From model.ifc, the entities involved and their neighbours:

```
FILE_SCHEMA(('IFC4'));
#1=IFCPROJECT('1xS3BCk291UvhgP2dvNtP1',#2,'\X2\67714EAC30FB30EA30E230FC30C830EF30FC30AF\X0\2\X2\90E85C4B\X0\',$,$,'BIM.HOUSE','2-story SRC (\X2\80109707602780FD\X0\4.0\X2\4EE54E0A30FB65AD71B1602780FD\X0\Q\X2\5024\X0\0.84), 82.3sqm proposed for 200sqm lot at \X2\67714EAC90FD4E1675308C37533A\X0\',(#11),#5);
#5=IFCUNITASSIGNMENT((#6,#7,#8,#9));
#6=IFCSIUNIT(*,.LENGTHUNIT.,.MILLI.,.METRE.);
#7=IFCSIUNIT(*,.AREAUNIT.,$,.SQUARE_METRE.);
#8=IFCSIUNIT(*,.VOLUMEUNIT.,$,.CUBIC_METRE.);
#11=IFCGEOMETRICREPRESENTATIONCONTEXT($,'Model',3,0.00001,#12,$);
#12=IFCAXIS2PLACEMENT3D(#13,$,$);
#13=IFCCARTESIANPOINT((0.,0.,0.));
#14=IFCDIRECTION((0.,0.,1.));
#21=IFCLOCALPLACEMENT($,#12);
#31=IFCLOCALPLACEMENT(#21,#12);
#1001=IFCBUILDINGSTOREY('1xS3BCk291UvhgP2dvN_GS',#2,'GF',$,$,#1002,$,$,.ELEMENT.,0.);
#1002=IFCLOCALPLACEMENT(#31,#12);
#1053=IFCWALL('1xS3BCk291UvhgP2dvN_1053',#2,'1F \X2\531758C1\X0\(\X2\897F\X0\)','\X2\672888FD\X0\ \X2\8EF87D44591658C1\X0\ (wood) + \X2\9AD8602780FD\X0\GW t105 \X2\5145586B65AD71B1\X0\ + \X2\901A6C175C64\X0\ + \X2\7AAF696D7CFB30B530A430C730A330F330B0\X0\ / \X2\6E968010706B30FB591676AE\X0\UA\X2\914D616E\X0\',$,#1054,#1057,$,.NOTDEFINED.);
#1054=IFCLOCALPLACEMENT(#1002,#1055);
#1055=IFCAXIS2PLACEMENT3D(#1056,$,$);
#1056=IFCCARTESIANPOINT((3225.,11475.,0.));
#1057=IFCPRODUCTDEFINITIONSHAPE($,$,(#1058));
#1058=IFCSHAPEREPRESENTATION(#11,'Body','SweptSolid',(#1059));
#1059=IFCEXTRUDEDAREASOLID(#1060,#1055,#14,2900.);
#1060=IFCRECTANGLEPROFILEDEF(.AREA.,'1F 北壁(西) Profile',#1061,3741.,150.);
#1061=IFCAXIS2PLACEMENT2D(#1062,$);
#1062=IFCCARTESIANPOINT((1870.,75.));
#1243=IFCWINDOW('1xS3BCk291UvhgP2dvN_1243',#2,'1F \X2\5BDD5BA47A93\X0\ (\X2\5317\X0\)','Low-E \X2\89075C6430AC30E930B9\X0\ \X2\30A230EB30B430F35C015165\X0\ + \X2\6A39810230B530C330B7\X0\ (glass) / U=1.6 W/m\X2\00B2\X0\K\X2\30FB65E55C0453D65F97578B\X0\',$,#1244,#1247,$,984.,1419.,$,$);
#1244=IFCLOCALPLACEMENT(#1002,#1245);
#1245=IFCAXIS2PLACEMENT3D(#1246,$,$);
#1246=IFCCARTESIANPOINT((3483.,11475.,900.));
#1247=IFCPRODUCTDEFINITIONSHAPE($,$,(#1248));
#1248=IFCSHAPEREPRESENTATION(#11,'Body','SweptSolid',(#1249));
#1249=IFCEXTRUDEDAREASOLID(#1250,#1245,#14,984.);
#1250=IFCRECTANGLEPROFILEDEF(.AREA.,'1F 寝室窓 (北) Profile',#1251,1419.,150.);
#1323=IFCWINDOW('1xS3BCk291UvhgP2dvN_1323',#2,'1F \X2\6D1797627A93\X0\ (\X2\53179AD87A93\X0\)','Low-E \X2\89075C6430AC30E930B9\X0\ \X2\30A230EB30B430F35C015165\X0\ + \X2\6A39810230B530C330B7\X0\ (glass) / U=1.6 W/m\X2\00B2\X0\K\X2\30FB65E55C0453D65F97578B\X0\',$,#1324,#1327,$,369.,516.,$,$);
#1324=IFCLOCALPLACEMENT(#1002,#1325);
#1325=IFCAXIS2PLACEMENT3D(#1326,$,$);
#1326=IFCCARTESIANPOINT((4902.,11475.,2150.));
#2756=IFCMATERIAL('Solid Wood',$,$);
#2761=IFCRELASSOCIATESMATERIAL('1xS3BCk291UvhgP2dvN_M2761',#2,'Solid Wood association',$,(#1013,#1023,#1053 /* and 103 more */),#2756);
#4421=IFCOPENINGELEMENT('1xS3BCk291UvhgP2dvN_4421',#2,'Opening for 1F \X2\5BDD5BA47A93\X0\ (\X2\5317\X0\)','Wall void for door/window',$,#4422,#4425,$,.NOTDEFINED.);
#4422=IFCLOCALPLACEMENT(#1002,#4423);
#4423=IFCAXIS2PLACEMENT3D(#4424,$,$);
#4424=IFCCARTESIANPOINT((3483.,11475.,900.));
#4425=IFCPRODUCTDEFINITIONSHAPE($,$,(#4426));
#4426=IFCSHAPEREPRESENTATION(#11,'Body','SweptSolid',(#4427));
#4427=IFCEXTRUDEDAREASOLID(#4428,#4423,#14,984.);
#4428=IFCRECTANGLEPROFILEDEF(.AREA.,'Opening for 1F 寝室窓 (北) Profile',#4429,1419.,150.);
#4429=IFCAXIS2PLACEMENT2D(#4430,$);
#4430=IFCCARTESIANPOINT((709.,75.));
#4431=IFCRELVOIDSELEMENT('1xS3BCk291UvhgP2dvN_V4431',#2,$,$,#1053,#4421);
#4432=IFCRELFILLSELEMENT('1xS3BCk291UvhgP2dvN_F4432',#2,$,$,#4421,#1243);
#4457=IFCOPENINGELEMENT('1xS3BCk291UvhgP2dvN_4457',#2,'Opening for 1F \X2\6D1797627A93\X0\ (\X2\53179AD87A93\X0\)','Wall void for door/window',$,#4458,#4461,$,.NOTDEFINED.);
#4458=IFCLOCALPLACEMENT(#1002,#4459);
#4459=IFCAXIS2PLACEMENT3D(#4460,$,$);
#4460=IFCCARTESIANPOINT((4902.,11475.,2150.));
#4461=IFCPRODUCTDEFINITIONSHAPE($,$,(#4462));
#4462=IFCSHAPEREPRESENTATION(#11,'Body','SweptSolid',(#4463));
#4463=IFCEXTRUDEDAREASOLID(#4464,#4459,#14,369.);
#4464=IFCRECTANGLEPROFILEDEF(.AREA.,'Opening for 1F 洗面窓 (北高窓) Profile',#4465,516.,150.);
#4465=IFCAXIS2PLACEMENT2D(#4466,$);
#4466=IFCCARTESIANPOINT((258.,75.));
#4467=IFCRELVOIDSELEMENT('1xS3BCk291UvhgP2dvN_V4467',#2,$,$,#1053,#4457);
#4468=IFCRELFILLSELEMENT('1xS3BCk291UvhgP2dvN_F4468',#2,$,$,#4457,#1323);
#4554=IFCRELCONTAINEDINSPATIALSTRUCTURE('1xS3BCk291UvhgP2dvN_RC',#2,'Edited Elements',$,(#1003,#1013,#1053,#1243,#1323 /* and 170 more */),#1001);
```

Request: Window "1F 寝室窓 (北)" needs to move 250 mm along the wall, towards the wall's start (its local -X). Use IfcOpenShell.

```python
import ifcopenshell
import ifcopenshell.api.geometry
import ifcopenshell.util.placement

model = ifcopenshell.open("model.ifc")

window = model.by_guid("1xS3BCk291UvhgP2dvN_1243")
opening = window.FillsVoids[0].RelatingOpeningElement
wall = opening.VoidsElements[0].RelatingBuildingElement

wall_matrix = ifcopenshell.util.placement.get_local_placement(wall.ObjectPlacement)
shift = wall_matrix[:3, 0] * -250.0
before = ifcopenshell.util.placement.get_local_placement(window.ObjectPlacement)[:3, 3].copy()

# The window is not placed relative to its opening, so move both.
for product in (opening, window):
    matrix = ifcopenshell.util.placement.get_local_placement(product.ObjectPlacement)
    matrix[:3, 3] += shift
    ifcopenshell.api.geometry.edit_object_placement(model, product=product, matrix=matrix, is_si=False)

after = ifcopenshell.util.placement.get_local_placement(window.ObjectPlacement)[:3, 3]
print("window moved by", (after - before).round(3) + 0.0)

model.write("model-out.ifc")
```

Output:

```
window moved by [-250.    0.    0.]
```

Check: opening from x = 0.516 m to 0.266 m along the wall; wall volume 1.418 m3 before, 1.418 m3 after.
